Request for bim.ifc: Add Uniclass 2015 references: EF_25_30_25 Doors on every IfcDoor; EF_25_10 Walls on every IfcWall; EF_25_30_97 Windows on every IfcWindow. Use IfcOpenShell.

First a look at what the model holds.

```python
import ifcopenshell

model = ifcopenshell.open("bim.ifc")
print(model.schema)
print("classifications:", [c.Name for c in model.by_type("IfcClassification")])
for ifc_class in ("IfcDoor", "IfcRoof", "IfcStair", "IfcWall", "IfcWindow"):
    print(ifc_class, len(model.by_type(ifc_class)))
```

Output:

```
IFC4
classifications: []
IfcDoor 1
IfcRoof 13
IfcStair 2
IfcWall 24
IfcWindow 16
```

```python
import ifcopenshell
import ifcopenshell.api.classification

model = ifcopenshell.open("bim.ifc")

system = ifcopenshell.api.classification.add_classification(model, classification="Uniclass 2015")

codes = {
    "IfcDoor": ("EF_25_30_25", "Doors"),
    "IfcWall": ("EF_25_10", "Walls"),
    "IfcWindow": ("EF_25_30_97", "Windows"),
}
for ifc_class, (code, name) in codes.items():
    products = model.by_type(ifc_class)
    ifcopenshell.api.classification.add_reference(
        model, products=products, classification=system, identification=code, name=name
    )
    print(code, len(products))

model.write("bim_v2.ifc")
```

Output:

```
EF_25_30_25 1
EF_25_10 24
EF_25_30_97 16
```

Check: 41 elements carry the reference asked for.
